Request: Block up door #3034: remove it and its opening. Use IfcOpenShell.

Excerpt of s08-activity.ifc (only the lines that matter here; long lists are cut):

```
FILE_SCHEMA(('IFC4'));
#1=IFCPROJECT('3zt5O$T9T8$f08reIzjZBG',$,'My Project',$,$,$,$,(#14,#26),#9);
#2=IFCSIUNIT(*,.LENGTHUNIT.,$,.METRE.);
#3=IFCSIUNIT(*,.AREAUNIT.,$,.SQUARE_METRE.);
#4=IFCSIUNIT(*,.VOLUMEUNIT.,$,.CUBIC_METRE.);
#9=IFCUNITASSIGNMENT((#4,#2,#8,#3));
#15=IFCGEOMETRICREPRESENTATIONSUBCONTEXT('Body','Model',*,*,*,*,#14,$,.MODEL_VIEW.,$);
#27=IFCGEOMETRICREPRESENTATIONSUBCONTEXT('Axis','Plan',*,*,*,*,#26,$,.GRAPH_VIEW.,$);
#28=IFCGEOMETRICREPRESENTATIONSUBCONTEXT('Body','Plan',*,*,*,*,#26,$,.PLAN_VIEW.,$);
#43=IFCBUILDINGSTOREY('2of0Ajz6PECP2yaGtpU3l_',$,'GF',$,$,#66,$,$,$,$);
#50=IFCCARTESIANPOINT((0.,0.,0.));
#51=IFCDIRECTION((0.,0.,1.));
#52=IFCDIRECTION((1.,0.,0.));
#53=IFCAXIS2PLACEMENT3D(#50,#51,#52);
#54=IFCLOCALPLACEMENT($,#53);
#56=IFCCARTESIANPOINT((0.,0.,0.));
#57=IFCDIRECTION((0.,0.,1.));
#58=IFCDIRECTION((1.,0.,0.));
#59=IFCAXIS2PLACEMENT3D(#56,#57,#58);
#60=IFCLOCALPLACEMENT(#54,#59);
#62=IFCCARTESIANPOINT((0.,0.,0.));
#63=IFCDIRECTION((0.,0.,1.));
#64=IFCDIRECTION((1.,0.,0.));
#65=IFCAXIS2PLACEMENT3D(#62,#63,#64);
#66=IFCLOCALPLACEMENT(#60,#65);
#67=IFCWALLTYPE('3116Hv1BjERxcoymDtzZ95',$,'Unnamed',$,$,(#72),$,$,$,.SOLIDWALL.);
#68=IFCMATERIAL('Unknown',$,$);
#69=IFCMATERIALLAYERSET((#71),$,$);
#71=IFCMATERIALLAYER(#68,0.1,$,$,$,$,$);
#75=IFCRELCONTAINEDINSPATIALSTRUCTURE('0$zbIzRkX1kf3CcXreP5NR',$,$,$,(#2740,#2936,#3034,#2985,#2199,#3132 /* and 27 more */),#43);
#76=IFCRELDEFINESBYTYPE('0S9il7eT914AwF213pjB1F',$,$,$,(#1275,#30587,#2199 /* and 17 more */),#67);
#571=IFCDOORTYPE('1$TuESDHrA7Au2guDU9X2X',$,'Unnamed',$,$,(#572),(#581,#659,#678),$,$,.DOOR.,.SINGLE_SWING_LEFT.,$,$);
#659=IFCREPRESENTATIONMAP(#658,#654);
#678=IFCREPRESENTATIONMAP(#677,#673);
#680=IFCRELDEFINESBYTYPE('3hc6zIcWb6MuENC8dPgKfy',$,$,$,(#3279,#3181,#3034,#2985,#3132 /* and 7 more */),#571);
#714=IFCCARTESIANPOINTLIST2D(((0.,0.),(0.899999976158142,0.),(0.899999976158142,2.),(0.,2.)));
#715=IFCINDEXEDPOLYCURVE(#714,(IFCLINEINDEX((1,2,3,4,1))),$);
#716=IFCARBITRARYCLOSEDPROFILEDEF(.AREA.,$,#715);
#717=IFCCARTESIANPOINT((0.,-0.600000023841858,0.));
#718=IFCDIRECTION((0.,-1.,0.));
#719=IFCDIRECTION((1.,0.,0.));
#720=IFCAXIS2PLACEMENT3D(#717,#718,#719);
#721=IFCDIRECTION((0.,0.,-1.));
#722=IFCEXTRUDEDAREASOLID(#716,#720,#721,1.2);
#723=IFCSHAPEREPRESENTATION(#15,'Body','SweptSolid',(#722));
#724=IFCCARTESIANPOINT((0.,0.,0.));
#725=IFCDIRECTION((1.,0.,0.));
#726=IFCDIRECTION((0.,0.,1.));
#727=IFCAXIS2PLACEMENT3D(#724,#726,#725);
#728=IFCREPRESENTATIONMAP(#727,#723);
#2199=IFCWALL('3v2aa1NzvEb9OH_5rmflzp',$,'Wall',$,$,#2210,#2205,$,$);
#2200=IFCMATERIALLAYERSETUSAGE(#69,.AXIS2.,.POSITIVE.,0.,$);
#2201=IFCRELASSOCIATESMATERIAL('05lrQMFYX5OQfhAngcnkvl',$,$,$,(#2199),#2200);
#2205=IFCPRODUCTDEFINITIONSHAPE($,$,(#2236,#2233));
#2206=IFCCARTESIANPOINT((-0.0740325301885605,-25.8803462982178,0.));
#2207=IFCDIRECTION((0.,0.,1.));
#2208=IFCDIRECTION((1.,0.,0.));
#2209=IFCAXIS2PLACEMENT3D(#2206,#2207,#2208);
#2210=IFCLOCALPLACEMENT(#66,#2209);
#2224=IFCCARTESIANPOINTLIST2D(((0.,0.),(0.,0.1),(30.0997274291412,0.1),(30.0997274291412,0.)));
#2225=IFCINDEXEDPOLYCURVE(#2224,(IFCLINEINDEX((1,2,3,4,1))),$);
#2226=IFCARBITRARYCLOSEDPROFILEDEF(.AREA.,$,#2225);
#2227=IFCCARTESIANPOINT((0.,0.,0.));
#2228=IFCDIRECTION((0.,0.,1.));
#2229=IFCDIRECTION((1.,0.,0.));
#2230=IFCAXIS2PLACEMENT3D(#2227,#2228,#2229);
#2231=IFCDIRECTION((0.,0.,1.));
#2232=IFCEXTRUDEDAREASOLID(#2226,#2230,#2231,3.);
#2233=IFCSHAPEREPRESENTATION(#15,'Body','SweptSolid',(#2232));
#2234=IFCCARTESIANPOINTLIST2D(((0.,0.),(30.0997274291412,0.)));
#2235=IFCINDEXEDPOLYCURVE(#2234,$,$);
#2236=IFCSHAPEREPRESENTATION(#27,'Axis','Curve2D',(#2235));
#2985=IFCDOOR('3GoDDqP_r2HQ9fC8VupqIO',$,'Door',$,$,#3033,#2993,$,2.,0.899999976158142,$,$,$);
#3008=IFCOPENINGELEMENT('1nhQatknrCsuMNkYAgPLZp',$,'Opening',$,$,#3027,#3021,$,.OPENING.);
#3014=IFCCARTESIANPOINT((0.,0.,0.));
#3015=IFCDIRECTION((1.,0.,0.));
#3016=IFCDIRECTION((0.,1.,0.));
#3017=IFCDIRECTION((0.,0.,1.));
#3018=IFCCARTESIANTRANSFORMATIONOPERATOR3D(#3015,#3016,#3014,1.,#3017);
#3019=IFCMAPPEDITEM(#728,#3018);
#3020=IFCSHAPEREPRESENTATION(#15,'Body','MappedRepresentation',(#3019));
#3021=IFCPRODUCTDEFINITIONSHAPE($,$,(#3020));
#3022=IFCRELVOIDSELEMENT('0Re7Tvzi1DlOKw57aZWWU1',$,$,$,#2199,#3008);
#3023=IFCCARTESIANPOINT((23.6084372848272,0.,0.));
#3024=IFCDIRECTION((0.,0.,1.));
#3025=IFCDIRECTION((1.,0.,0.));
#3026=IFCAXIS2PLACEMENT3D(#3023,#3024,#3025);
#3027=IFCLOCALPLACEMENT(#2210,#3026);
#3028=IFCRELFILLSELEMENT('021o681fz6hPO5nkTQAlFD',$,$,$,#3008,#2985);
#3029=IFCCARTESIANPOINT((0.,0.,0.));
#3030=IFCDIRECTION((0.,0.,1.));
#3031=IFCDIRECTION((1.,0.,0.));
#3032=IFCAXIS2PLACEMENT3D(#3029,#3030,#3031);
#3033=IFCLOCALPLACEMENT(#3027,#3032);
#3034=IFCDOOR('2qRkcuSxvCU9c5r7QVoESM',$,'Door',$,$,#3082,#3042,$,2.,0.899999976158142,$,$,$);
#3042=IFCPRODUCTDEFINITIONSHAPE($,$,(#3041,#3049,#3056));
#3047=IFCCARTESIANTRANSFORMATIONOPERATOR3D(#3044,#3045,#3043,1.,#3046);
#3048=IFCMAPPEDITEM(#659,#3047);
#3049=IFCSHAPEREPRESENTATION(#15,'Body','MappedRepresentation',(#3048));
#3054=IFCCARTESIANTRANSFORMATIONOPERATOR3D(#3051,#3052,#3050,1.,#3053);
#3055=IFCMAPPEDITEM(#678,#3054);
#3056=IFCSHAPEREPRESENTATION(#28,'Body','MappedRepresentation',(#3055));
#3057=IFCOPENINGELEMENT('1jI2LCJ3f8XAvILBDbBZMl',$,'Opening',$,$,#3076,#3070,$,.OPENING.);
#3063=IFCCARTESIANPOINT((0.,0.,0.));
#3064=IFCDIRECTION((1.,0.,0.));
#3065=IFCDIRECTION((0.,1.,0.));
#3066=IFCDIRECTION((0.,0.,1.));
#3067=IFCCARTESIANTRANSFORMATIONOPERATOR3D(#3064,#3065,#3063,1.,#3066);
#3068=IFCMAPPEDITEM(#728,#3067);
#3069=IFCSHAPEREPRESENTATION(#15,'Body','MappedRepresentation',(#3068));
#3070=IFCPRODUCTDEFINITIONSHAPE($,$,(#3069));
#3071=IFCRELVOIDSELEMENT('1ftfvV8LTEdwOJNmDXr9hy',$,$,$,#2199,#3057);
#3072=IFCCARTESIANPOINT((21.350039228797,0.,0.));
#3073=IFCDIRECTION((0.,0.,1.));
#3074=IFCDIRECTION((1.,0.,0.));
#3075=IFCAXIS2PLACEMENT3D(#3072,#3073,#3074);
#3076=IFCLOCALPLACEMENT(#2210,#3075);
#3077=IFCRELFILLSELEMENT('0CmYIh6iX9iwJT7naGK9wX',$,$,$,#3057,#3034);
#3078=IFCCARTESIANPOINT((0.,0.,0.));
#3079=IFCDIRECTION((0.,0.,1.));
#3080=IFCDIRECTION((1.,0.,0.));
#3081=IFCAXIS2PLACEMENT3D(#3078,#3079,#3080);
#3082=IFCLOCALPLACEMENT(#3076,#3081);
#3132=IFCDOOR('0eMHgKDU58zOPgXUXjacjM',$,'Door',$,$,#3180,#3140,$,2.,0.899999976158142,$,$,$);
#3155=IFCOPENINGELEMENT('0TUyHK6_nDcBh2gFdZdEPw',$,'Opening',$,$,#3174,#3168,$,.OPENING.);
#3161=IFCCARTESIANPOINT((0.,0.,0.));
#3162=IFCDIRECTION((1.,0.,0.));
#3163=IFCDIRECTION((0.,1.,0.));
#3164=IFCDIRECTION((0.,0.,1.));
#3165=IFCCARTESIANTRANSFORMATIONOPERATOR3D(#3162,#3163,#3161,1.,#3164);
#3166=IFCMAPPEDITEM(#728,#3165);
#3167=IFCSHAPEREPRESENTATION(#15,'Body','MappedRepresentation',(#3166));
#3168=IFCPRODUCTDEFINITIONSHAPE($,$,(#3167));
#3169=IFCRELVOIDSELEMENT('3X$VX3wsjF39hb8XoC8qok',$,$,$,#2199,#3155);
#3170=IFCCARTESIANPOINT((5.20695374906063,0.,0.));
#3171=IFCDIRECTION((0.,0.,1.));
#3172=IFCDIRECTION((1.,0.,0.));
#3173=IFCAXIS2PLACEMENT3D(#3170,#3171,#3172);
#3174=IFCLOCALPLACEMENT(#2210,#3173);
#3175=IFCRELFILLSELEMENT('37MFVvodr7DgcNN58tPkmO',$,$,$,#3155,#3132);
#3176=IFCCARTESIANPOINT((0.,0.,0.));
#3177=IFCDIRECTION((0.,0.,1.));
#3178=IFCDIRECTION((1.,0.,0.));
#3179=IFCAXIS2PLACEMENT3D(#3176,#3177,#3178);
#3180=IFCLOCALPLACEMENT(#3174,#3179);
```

```python
import ifcopenshell
import ifcopenshell.api.feature
import ifcopenshell.api.root
import ifcopenshell.geom
import ifcopenshell.util.shape

model = ifcopenshell.open("s08-activity.ifc")
settings = ifcopenshell.geom.settings()


def volume(element):
    """Net volume in cubic metres, openings subtracted."""
    shape = ifcopenshell.geom.create_shape(settings, element)
    return ifcopenshell.util.shape.get_volume(shape.geometry)


door = model.by_guid("2qRkcuSxvCU9c5r7QVoESM")
opening = door.FillsVoids[0].RelatingOpeningElement
wall = opening.VoidsElements[0].RelatingBuildingElement
before = volume(wall)

ifcopenshell.api.root.remove_product(model, product=door)
ifcopenshell.api.feature.remove_feature(model, feature=opening)

after = volume(wall)

print(f"wall volume {before:.3f} -> {after:.3f} m3")

model.write("s08-activity_v2.ifc")
```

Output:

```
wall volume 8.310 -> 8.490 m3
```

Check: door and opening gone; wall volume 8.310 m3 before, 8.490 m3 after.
